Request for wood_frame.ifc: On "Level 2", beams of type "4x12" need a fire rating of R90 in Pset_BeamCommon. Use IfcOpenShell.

First a look at what the model holds.

```python
import ifcopenshell
import ifcopenshell.util.element

model = ifcopenshell.open("wood_frame.ifc")
print(model.schema)
storey = next(s for s in model.by_type("IfcBuildingStorey") if s.Name == "Level 2")
beams = [e for e in ifcopenshell.util.element.get_decomposition(storey) if e.is_a("IfcBeam")]
seen = {}
for e in beams:
    element_type = ifcopenshell.util.element.get_type(e)
    key = (element_type.Name if element_type != e and element_type else None, ifcopenshell.util.element.get_pset(e, "Pset_BeamCommon", "FireRating"))
    seen[key] = seen.get(key, 0) + 1
for (name, value), count in sorted(seen.items(), key=str):
    print(count, "x", name, "|", value)
```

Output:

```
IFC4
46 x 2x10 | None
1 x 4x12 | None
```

```python
import ifcopenshell
import ifcopenshell.api.pset
import ifcopenshell.util.element

model = ifcopenshell.open("wood_frame.ifc")

storey = next(s for s in model.by_type("IfcBuildingStorey") if s.Name == "Level 2")
beams = [e for e in ifcopenshell.util.element.get_decomposition(storey) if e.is_a("IfcBeam")]

count = 0
for e in beams:
    element_type = ifcopenshell.util.element.get_type(e)
    if element_type in (None, e) or element_type.Name != "4x12":
        continue
    # add_pset returns the element's existing set when there is one.
    pset = ifcopenshell.api.pset.add_pset(model, product=e, name="Pset_BeamCommon")
    ifcopenshell.api.pset.edit_pset(model, pset=pset, properties={"FireRating": "R90"})
    count += 1

print(count, "beams updated")

model.write("wood_frame_updated.ifc")
```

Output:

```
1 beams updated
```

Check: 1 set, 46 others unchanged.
